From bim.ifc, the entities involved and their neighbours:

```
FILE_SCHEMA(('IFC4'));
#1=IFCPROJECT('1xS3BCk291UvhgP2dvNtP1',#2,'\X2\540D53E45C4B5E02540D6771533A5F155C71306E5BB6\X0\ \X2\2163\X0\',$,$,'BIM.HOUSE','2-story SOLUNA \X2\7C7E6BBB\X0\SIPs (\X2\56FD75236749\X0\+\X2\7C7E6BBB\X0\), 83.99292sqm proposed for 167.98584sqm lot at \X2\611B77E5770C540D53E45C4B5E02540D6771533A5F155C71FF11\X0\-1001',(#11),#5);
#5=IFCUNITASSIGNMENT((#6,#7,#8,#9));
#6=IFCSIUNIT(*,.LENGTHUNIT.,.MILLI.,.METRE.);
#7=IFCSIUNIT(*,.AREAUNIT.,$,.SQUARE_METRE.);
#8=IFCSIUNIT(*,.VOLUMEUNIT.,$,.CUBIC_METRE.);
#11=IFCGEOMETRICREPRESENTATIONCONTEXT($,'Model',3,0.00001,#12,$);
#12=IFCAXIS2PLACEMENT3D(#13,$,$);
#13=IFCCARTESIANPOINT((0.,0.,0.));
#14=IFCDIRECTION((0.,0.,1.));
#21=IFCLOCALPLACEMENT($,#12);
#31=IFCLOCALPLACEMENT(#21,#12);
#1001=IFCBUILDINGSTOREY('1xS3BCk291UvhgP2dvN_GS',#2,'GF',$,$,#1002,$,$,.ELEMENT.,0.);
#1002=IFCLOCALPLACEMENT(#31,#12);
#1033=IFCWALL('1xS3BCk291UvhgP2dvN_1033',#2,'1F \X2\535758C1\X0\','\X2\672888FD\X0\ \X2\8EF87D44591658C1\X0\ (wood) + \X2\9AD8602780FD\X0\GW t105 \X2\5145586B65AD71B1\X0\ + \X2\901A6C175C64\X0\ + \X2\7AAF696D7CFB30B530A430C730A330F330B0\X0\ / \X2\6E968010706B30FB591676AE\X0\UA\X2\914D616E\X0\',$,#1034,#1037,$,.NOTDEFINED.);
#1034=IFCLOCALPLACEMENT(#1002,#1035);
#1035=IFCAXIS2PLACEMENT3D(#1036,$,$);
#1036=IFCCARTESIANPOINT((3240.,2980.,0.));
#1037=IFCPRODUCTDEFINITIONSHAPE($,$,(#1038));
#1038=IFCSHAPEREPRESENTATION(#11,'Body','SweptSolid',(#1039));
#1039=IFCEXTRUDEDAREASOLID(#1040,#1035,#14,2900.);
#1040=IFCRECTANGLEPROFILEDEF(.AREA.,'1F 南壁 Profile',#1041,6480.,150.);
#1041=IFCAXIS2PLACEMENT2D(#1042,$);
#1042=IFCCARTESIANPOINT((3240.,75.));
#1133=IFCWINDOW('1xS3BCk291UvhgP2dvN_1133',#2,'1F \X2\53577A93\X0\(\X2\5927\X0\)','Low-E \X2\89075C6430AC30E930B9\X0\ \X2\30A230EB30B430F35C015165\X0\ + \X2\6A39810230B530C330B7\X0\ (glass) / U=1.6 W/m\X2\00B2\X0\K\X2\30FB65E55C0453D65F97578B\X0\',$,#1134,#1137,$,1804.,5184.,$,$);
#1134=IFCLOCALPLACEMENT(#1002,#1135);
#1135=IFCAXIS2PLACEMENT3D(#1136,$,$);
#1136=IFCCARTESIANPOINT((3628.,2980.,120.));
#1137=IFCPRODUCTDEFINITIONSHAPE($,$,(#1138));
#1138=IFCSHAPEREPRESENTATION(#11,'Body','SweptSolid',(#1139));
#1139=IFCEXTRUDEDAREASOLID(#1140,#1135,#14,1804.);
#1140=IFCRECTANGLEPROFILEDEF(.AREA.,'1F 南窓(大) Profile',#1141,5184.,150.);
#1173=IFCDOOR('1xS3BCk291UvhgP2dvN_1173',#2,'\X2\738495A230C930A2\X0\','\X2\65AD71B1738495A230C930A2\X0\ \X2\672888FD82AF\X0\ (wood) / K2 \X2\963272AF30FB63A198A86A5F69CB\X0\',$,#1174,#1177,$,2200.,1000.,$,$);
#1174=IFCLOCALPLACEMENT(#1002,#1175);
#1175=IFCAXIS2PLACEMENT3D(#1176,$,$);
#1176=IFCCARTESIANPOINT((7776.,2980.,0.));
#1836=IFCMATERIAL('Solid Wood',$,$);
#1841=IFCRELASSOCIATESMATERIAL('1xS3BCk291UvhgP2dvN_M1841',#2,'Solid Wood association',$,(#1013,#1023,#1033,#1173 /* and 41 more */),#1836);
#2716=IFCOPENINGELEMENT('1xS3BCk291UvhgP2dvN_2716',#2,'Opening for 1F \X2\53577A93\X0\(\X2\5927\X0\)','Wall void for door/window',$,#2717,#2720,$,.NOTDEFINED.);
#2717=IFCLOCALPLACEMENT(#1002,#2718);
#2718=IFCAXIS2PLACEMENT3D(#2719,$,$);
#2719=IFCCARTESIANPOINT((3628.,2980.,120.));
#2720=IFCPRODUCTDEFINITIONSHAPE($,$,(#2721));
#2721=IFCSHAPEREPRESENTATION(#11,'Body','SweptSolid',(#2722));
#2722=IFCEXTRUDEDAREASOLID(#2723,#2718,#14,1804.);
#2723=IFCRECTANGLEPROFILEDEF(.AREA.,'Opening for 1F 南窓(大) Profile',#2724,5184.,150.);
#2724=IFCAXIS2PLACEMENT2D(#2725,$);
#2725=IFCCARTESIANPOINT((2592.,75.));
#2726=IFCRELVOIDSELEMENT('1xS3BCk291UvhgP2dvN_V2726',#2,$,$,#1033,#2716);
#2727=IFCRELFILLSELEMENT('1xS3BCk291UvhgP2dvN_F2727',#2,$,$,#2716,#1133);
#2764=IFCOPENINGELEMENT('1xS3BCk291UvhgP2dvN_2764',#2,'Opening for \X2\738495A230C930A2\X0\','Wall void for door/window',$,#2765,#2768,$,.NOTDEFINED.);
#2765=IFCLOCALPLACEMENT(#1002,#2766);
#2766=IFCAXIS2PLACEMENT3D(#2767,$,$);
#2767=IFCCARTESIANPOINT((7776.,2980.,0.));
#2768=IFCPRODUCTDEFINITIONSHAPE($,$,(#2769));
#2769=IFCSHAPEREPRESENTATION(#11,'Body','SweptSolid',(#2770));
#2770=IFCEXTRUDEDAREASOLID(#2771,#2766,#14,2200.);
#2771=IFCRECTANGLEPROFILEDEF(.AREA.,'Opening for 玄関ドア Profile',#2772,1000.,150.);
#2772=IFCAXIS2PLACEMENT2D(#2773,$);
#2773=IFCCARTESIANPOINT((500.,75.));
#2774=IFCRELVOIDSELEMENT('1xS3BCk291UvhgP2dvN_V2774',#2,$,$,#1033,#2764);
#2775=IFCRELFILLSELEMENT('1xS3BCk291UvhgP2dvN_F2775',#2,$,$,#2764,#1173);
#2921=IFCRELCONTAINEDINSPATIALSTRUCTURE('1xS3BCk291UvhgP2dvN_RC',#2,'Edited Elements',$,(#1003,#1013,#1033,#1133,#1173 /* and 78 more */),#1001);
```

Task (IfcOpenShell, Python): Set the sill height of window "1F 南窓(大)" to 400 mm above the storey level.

```python
import numpy as np
import ifcopenshell
import ifcopenshell.api.geometry
import ifcopenshell.geom
import ifcopenshell.util.element
import ifcopenshell.util.placement
import ifcopenshell.util.shape
import ifcopenshell.util.unit

model = ifcopenshell.open("bim.ifc")
unit_scale = ifcopenshell.util.unit.calculate_unit_scale(model)

window = model.by_guid("1xS3BCk291UvhgP2dvN_1133")
opening = window.FillsVoids[0].RelatingOpeningElement
storey = ifcopenshell.util.element.get_container(window, ifc_class="IfcBuildingStorey")
level = ifcopenshell.util.placement.get_local_placement(storey.ObjectPlacement)[2, 3]

# The opening's origin need not be at the sill, so measure its lowest point.
shape = ifcopenshell.geom.create_shape(ifcopenshell.geom.settings(), opening)
bottom = ifcopenshell.util.shape.get_shape_bottom_elevation(shape, shape.geometry) / unit_scale
dz = level + 400.0 - bottom

shift = np.array([0.0, 0.0, dz])
# The window is not placed relative to its opening, so move both.
for product in (opening, window):
    matrix = ifcopenshell.util.placement.get_local_placement(product.ObjectPlacement)
    matrix[:3, 3] += shift
    ifcopenshell.api.geometry.edit_object_placement(model, product=product, matrix=matrix, is_si=False)

print(f"moved by {dz * unit_scale:+.3f} m")

model.write("bim_updated.ifc")
```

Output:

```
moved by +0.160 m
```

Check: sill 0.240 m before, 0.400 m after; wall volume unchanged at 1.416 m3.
